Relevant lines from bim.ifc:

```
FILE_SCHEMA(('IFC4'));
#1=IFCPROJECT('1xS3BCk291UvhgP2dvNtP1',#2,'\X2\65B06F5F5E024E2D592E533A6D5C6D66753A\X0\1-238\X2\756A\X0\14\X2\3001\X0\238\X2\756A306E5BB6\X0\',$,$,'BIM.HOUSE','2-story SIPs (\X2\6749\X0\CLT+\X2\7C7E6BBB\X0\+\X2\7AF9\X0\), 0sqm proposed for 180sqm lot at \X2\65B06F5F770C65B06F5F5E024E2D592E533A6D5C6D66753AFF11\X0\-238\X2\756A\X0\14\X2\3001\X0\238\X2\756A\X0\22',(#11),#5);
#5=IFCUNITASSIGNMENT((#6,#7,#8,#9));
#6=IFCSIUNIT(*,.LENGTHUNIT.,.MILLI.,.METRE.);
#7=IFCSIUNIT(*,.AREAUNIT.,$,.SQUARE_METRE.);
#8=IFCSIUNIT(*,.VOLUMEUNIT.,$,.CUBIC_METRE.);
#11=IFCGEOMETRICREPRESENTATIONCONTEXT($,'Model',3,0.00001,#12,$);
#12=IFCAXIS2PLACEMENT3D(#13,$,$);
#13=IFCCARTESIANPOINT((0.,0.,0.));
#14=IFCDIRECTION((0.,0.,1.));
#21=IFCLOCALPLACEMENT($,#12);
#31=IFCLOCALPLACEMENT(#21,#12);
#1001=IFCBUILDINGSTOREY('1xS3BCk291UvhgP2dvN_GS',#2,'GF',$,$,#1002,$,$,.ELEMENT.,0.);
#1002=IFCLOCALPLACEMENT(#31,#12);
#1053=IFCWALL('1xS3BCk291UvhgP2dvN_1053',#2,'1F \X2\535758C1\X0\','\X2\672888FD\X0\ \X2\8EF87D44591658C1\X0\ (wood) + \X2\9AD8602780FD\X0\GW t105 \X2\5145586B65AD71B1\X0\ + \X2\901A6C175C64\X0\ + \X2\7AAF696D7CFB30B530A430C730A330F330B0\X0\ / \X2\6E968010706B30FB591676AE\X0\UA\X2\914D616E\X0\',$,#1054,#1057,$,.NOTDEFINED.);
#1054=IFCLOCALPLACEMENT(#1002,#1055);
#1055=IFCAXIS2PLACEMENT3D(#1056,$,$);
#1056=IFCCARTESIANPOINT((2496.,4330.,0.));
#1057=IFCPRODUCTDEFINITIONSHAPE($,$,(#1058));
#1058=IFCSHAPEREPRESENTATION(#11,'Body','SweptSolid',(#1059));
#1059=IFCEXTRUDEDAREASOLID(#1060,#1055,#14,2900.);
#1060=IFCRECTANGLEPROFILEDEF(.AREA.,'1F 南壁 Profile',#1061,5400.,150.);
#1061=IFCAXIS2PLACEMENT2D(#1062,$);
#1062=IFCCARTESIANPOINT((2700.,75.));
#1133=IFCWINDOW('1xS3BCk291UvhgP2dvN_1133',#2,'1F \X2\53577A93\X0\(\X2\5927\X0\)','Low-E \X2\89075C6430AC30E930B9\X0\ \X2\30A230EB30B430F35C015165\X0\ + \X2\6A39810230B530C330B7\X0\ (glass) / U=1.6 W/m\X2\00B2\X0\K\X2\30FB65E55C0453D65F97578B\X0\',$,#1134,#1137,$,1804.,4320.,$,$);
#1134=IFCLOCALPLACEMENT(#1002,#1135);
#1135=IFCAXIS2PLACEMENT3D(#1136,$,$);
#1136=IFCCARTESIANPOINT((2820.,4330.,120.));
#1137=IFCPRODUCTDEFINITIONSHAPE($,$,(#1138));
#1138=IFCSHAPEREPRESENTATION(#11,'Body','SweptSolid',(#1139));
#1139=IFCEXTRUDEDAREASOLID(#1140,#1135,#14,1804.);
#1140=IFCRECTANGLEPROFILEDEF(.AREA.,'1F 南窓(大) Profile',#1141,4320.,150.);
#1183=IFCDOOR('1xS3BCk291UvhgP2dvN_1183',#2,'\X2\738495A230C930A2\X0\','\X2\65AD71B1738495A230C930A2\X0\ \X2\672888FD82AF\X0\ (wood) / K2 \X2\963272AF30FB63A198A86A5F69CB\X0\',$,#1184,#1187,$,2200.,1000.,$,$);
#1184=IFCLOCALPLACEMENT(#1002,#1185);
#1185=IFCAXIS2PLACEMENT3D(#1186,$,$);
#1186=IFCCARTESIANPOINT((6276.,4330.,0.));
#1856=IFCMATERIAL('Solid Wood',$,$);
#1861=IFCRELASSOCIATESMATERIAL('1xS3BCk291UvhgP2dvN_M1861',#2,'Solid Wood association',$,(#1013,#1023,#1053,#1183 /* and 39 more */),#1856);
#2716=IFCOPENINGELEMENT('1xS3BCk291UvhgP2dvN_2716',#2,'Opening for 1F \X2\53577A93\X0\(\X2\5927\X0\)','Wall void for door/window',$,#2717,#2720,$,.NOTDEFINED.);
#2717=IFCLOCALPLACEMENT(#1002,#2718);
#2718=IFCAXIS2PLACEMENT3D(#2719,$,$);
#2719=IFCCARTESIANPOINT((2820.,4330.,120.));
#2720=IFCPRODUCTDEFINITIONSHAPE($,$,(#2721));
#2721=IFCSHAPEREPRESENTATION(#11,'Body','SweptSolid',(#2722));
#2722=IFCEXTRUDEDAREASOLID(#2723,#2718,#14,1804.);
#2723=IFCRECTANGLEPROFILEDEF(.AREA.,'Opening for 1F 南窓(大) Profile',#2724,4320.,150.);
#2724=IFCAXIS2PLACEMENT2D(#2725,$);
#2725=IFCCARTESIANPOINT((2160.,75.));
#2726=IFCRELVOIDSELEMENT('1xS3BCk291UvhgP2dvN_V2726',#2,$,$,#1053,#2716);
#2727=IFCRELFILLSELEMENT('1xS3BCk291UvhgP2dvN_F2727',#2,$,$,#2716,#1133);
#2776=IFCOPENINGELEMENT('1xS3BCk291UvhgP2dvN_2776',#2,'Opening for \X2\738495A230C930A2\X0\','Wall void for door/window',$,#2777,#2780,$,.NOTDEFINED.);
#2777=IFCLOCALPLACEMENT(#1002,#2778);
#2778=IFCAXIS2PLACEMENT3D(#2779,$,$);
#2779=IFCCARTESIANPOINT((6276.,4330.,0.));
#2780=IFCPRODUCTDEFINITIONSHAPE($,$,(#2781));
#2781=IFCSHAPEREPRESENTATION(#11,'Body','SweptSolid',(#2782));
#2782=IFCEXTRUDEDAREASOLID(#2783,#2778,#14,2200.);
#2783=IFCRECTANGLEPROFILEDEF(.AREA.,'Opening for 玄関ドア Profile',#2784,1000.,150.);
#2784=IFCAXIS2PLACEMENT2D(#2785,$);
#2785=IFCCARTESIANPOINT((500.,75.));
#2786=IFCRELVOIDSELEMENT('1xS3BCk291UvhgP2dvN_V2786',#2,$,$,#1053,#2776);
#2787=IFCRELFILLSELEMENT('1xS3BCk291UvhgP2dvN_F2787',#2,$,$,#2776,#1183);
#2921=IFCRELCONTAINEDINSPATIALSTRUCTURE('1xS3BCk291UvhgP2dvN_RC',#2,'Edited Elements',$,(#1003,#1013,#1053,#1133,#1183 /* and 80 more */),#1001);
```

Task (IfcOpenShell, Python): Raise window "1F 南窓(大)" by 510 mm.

```python
import numpy as np
import ifcopenshell
import ifcopenshell.api.geometry
import ifcopenshell.util.placement
import ifcopenshell.util.unit

model = ifcopenshell.open("bim.ifc")
unit_scale = ifcopenshell.util.unit.calculate_unit_scale(model)

window = model.by_id(1133)
opening = window.FillsVoids[0].RelatingOpeningElement
dz = 0.51 / unit_scale

shift = np.array([0.0, 0.0, dz])
# The window is not placed relative to its opening, so move both.
for product in (opening, window):
    matrix = ifcopenshell.util.placement.get_local_placement(product.ObjectPlacement)
    matrix[:3, 3] += shift
    ifcopenshell.api.geometry.edit_object_placement(model, product=product, matrix=matrix, is_si=False)

print(f"moved by {dz * unit_scale:+.3f} m")

model.write("bim-out.ifc")
```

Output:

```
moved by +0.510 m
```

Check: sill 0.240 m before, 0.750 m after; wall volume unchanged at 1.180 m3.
